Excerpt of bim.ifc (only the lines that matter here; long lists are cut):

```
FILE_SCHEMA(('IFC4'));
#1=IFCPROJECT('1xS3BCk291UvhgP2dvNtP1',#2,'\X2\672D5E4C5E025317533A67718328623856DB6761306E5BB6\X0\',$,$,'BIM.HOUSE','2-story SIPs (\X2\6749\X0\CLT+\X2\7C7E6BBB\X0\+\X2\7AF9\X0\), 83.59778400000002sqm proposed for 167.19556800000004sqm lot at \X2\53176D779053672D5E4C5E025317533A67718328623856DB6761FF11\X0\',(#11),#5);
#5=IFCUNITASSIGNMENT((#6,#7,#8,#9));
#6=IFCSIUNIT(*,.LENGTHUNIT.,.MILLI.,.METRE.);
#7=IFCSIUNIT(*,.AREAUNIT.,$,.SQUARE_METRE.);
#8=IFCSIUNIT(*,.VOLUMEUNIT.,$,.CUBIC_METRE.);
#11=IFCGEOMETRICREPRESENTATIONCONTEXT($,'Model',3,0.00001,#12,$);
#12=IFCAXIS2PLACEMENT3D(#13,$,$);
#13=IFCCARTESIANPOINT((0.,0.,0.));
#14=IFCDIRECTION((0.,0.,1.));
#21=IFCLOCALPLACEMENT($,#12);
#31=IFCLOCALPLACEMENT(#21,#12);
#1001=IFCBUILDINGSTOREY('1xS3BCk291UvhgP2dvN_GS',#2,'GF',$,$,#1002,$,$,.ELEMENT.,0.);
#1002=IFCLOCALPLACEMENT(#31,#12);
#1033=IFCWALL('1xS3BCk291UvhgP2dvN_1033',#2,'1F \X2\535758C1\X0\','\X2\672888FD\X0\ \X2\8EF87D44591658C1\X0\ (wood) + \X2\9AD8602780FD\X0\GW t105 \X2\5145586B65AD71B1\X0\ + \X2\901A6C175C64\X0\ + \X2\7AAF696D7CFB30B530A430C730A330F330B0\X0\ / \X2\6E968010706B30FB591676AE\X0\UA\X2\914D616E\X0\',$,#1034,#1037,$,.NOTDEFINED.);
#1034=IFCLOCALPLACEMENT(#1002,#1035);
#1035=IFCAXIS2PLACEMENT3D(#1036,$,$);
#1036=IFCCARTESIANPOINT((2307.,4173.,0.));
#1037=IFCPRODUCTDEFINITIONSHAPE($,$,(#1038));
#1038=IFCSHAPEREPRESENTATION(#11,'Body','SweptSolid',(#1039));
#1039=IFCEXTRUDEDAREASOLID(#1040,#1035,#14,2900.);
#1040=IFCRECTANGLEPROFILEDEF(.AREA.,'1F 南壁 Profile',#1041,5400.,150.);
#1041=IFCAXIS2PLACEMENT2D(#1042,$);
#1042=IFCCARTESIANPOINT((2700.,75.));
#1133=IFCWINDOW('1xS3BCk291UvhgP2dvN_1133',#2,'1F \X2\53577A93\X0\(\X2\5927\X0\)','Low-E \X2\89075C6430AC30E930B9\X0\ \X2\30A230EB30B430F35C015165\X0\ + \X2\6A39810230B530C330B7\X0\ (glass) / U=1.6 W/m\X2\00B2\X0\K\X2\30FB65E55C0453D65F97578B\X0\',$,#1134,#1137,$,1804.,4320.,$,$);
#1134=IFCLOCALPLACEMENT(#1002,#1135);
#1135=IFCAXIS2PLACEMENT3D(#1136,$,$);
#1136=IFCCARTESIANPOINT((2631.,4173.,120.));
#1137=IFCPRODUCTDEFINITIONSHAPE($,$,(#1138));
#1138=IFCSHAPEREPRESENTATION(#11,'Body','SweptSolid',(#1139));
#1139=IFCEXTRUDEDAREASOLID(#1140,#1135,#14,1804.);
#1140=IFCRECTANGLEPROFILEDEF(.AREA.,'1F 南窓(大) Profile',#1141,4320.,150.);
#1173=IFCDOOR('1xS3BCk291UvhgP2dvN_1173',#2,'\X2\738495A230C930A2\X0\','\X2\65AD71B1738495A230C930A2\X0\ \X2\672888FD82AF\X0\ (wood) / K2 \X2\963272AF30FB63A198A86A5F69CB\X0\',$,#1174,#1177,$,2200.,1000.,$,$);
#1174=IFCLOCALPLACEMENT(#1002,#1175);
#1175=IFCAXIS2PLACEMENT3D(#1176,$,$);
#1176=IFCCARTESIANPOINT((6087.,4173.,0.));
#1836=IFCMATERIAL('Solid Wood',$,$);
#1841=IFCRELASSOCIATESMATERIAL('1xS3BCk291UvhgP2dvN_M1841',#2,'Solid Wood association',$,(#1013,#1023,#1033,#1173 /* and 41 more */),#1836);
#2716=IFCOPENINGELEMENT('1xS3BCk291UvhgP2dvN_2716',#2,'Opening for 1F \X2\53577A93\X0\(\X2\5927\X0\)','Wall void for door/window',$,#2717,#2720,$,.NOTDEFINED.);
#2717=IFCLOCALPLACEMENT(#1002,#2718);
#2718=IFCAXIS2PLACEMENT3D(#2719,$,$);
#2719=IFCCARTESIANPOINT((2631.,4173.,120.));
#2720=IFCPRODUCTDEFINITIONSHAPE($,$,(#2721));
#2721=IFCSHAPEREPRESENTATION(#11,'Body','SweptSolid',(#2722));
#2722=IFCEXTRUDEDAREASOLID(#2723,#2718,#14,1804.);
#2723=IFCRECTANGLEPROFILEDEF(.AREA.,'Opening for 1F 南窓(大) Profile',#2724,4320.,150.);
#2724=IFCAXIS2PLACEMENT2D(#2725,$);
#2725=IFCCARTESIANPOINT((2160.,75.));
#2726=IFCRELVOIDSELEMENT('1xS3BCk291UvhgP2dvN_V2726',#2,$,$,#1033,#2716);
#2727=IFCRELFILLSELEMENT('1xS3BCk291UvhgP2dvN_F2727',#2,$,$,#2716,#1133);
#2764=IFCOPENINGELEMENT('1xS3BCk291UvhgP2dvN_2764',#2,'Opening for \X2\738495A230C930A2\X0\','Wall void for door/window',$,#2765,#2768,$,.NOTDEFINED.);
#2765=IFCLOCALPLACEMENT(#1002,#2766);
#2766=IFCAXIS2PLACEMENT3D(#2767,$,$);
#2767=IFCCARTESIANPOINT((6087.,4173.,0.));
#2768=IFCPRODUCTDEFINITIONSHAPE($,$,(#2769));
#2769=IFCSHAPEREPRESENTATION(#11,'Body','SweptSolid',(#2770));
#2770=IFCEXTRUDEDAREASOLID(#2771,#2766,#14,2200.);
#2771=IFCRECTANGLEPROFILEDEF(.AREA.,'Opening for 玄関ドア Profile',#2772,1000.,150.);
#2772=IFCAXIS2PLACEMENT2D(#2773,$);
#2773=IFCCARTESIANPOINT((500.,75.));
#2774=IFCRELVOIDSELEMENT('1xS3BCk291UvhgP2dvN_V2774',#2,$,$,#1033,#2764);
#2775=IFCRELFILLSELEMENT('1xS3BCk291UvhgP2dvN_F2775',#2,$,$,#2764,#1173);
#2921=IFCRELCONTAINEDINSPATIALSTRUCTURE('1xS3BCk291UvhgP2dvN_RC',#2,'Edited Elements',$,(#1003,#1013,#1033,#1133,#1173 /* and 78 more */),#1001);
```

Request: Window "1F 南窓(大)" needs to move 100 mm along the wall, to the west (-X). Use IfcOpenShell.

```python
import ifcopenshell
import ifcopenshell.api.geometry
import ifcopenshell.util.placement

model = ifcopenshell.open("bim.ifc")

window = model.by_guid("1xS3BCk291UvhgP2dvN_1133")
opening = window.FillsVoids[0].RelatingOpeningElement
wall = opening.VoidsElements[0].RelatingBuildingElement

wall_matrix = ifcopenshell.util.placement.get_local_placement(wall.ObjectPlacement)
shift = wall_matrix[:3, 0] * -100.0
before = ifcopenshell.util.placement.get_local_placement(window.ObjectPlacement)[:3, 3].copy()

# The window is not placed relative to its opening, so move both.
for product in (opening, window):
    matrix = ifcopenshell.util.placement.get_local_placement(product.ObjectPlacement)
    matrix[:3, 3] += shift
    ifcopenshell.api.geometry.edit_object_placement(model, product=product, matrix=matrix, is_si=False)

after = ifcopenshell.util.placement.get_local_placement(window.ObjectPlacement)[:3, 3]
print("window moved by", (after - before).round(3) + 0.0)

model.write("bim_edited.ifc")
```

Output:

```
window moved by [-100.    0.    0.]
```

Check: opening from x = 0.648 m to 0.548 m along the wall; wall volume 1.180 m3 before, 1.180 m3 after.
